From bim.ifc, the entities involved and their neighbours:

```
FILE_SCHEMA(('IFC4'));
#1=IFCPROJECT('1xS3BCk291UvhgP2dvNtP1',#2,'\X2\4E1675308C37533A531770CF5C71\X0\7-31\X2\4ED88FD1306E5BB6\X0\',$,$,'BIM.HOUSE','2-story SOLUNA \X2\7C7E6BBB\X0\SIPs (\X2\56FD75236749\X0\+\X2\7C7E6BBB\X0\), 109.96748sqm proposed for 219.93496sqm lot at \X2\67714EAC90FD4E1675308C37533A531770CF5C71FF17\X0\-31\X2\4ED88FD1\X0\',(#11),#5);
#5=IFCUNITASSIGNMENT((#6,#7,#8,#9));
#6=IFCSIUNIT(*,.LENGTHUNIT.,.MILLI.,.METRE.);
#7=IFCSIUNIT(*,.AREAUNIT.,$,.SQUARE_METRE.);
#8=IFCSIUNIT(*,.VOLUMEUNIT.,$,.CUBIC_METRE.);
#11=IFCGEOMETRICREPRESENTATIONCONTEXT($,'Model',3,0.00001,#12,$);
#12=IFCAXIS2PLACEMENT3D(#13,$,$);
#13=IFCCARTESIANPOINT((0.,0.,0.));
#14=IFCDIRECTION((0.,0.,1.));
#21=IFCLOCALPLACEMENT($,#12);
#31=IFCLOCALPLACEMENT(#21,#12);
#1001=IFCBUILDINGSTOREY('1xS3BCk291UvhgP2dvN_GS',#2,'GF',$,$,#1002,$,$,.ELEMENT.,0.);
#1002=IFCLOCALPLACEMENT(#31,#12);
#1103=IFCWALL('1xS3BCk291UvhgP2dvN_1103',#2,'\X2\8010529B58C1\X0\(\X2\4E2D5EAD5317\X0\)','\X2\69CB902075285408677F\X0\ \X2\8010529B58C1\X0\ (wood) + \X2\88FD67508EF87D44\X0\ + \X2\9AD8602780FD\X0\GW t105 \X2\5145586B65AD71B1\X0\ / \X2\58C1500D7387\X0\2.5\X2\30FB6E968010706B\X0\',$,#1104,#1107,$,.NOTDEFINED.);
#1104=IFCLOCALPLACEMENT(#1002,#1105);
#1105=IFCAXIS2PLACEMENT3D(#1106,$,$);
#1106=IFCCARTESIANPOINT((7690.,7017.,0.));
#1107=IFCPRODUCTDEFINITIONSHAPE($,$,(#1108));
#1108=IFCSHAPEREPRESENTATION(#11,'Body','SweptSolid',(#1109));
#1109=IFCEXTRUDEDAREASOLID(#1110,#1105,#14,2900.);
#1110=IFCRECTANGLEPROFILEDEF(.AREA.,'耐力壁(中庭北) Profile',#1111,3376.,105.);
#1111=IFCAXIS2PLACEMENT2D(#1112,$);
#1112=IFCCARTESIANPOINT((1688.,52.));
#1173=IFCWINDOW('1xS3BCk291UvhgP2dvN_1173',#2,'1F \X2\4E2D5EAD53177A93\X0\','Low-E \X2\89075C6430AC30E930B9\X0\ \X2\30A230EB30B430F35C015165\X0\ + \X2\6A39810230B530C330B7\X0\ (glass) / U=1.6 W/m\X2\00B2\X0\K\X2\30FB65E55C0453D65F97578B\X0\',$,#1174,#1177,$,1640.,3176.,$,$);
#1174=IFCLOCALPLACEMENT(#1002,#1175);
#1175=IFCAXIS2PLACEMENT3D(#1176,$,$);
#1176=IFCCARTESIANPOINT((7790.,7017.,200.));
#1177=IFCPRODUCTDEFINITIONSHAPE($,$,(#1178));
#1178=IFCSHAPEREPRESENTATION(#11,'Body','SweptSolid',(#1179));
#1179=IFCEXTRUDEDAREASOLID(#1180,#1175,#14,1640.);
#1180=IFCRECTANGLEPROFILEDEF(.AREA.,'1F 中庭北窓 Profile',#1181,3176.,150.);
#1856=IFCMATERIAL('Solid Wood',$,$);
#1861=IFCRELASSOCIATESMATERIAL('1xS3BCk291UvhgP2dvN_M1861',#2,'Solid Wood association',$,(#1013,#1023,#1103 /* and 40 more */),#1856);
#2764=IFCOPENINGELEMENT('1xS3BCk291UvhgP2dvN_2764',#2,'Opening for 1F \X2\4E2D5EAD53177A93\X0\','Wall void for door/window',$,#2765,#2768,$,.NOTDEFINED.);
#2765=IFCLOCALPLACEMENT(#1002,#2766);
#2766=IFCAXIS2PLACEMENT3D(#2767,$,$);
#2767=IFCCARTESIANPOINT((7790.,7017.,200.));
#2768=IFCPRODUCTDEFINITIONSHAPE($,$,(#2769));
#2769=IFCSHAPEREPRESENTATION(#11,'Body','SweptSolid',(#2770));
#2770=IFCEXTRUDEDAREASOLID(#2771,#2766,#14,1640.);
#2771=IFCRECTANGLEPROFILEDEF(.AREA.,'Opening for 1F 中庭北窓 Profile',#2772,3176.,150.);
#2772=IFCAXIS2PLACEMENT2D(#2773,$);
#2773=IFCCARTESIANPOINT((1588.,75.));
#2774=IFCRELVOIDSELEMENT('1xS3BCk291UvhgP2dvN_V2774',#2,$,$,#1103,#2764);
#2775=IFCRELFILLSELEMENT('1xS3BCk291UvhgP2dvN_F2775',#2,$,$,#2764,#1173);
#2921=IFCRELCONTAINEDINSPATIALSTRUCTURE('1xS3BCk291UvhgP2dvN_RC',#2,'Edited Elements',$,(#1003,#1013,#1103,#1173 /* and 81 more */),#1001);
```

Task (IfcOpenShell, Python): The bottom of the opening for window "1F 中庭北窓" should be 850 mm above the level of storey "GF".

```python
import numpy as np
import ifcopenshell
import ifcopenshell.api.geometry
import ifcopenshell.geom
import ifcopenshell.util.element
import ifcopenshell.util.placement
import ifcopenshell.util.shape
import ifcopenshell.util.unit

model = ifcopenshell.open("bim.ifc")
unit_scale = ifcopenshell.util.unit.calculate_unit_scale(model)

window = model.by_guid("1xS3BCk291UvhgP2dvN_1173")
opening = window.FillsVoids[0].RelatingOpeningElement
storey = ifcopenshell.util.element.get_container(window, ifc_class="IfcBuildingStorey")
level = ifcopenshell.util.placement.get_local_placement(storey.ObjectPlacement)[2, 3]

# The opening's origin need not be at the sill, so measure its lowest point.
shape = ifcopenshell.geom.create_shape(ifcopenshell.geom.settings(), opening)
bottom = ifcopenshell.util.shape.get_shape_bottom_elevation(shape, shape.geometry) / unit_scale
dz = level + 0.85 / unit_scale - bottom

shift = np.array([0.0, 0.0, dz])
# The window is not placed relative to its opening, so move both.
for product in (opening, window):
    matrix = ifcopenshell.util.placement.get_local_placement(product.ObjectPlacement)
    matrix[:3, 3] += shift
    ifcopenshell.api.geometry.edit_object_placement(model, product=product, matrix=matrix, is_si=False)

print(f"moved by {dz * unit_scale:+.3f} m")

model.write("bim_updated.ifc")
```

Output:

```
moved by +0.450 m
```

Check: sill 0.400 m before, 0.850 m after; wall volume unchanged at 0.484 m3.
